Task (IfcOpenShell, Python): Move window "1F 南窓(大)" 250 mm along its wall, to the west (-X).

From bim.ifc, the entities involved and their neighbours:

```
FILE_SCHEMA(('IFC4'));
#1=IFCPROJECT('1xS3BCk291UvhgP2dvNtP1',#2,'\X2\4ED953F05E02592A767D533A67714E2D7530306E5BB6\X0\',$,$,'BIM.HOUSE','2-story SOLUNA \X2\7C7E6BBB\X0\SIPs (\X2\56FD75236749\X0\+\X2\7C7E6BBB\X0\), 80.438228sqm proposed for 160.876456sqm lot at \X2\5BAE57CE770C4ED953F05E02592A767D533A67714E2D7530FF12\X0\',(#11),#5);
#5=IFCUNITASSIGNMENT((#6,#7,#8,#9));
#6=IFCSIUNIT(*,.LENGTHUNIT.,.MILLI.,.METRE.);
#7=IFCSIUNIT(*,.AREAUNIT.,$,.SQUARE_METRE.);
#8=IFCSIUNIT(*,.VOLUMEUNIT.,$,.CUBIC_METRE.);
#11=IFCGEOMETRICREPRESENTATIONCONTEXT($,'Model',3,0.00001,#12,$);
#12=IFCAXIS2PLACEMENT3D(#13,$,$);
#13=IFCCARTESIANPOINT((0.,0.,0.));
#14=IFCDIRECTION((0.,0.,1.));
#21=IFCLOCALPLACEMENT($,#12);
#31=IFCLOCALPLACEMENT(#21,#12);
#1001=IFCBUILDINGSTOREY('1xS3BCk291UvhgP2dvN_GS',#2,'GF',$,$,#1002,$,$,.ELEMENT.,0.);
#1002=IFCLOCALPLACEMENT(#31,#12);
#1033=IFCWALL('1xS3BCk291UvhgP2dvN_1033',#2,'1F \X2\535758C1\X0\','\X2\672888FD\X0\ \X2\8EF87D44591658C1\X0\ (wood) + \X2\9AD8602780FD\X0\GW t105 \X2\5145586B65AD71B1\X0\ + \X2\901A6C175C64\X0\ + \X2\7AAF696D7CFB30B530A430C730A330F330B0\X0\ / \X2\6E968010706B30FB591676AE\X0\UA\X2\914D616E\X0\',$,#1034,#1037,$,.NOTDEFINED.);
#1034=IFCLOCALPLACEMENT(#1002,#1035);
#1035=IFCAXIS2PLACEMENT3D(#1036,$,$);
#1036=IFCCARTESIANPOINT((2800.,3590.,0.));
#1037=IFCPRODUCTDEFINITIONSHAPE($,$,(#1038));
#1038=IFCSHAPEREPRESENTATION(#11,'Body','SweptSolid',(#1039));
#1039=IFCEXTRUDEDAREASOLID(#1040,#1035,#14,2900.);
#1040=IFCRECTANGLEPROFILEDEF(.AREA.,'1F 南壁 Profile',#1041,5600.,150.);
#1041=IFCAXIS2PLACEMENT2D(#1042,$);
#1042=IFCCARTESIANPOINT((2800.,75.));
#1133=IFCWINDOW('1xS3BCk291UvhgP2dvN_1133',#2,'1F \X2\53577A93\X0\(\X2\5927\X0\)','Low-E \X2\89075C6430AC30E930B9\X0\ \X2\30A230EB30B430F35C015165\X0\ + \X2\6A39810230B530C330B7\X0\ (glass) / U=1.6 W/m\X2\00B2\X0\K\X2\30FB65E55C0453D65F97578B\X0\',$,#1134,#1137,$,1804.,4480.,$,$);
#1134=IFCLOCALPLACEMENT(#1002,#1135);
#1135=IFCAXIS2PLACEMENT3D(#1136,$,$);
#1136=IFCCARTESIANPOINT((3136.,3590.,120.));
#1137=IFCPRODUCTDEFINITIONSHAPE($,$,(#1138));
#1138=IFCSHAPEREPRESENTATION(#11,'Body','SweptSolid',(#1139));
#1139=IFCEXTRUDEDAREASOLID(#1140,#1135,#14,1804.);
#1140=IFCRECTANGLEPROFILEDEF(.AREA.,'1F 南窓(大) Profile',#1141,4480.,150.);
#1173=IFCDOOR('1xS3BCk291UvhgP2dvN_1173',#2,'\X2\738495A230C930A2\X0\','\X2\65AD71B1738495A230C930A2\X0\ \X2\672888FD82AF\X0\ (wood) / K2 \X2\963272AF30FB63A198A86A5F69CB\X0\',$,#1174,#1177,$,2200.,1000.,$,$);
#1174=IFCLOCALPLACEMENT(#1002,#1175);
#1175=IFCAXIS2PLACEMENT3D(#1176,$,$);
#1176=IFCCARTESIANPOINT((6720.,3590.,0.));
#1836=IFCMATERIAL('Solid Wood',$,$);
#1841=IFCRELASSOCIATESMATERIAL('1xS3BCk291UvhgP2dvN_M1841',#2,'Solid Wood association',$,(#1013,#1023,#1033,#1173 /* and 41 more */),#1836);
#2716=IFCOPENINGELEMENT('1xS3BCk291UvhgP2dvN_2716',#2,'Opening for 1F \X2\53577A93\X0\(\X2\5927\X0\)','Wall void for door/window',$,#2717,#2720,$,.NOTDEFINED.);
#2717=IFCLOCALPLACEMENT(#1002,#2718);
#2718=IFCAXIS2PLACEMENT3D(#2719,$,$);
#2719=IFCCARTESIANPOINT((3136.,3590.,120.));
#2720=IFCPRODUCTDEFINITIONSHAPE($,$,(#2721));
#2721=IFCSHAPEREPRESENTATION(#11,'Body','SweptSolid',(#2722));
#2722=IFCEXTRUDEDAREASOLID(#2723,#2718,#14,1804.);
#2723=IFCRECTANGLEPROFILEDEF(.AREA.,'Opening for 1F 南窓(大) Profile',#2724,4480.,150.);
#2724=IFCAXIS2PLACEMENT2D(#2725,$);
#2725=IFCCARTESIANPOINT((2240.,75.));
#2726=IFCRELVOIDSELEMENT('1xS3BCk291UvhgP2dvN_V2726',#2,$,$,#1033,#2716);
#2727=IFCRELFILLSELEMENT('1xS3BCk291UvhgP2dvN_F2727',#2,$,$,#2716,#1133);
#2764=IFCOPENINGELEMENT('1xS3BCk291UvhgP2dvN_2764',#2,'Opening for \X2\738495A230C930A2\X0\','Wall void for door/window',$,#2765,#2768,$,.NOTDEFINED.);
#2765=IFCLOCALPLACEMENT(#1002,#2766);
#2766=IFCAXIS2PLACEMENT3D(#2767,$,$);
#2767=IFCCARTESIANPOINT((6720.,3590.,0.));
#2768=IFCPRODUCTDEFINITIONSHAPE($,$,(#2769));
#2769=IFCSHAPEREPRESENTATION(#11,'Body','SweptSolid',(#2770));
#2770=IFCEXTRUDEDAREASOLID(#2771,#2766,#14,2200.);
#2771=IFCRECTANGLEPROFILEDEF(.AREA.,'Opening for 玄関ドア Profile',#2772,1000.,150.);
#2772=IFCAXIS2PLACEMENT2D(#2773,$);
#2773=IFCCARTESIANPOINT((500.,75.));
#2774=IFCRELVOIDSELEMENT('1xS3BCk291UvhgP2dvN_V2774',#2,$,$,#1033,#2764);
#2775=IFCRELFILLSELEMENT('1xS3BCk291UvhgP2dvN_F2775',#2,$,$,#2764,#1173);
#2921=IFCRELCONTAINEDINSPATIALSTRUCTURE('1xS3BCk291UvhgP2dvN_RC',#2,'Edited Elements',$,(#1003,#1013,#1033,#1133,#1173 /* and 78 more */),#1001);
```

```python
import ifcopenshell
import ifcopenshell.api.geometry
import ifcopenshell.util.placement
import ifcopenshell.util.unit

model = ifcopenshell.open("bim.ifc")
unit_scale = ifcopenshell.util.unit.calculate_unit_scale(model)

window = model.by_guid("1xS3BCk291UvhgP2dvN_1133")
opening = window.FillsVoids[0].RelatingOpeningElement
wall = opening.VoidsElements[0].RelatingBuildingElement

wall_matrix = ifcopenshell.util.placement.get_local_placement(wall.ObjectPlacement)
shift = wall_matrix[:3, 0] * -0.25 / unit_scale
before = ifcopenshell.util.placement.get_local_placement(window.ObjectPlacement)[:3, 3].copy()

# The window is not placed relative to its opening, so move both.
for product in (opening, window):
    matrix = ifcopenshell.util.placement.get_local_placement(product.ObjectPlacement)
    matrix[:3, 3] += shift
    ifcopenshell.api.geometry.edit_object_placement(model, product=product, matrix=matrix, is_si=False)

after = ifcopenshell.util.placement.get_local_placement(window.ObjectPlacement)[:3, 3]
print("window moved by", (after - before).round(3) + 0.0)

model.write("bim_v2.ifc")
```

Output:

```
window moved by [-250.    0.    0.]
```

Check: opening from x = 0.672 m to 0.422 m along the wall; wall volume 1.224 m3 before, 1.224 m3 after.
